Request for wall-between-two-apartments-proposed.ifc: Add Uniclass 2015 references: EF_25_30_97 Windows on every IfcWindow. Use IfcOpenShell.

First a look at what the model holds.

```python
import ifcopenshell

model = ifcopenshell.open("wall-between-two-apartments-proposed.ifc")
print(model.schema)
print("classifications:", [c.Name for c in model.by_type("IfcClassification")])
for ifc_class in ("IfcDoor", "IfcRoof", "IfcStair", "IfcWall", "IfcWindow"):
    print(ifc_class, len(model.by_type(ifc_class)))
```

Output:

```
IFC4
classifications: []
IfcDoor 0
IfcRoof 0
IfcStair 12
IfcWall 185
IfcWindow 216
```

```python
import ifcopenshell
import ifcopenshell.api.classification

model = ifcopenshell.open("wall-between-two-apartments-proposed.ifc")

system = ifcopenshell.api.classification.add_classification(model, classification="Uniclass 2015")

codes = {
    "IfcWindow": ("EF_25_30_97", "Windows"),
}
for ifc_class, (code, name) in codes.items():
    products = model.by_type(ifc_class)
    ifcopenshell.api.classification.add_reference(
        model, products=products, classification=system, identification=code, name=name
    )
    print(code, len(products))

model.write("wall-between-two-apartments-proposed_updated.ifc")
```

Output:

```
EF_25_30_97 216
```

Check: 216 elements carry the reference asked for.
